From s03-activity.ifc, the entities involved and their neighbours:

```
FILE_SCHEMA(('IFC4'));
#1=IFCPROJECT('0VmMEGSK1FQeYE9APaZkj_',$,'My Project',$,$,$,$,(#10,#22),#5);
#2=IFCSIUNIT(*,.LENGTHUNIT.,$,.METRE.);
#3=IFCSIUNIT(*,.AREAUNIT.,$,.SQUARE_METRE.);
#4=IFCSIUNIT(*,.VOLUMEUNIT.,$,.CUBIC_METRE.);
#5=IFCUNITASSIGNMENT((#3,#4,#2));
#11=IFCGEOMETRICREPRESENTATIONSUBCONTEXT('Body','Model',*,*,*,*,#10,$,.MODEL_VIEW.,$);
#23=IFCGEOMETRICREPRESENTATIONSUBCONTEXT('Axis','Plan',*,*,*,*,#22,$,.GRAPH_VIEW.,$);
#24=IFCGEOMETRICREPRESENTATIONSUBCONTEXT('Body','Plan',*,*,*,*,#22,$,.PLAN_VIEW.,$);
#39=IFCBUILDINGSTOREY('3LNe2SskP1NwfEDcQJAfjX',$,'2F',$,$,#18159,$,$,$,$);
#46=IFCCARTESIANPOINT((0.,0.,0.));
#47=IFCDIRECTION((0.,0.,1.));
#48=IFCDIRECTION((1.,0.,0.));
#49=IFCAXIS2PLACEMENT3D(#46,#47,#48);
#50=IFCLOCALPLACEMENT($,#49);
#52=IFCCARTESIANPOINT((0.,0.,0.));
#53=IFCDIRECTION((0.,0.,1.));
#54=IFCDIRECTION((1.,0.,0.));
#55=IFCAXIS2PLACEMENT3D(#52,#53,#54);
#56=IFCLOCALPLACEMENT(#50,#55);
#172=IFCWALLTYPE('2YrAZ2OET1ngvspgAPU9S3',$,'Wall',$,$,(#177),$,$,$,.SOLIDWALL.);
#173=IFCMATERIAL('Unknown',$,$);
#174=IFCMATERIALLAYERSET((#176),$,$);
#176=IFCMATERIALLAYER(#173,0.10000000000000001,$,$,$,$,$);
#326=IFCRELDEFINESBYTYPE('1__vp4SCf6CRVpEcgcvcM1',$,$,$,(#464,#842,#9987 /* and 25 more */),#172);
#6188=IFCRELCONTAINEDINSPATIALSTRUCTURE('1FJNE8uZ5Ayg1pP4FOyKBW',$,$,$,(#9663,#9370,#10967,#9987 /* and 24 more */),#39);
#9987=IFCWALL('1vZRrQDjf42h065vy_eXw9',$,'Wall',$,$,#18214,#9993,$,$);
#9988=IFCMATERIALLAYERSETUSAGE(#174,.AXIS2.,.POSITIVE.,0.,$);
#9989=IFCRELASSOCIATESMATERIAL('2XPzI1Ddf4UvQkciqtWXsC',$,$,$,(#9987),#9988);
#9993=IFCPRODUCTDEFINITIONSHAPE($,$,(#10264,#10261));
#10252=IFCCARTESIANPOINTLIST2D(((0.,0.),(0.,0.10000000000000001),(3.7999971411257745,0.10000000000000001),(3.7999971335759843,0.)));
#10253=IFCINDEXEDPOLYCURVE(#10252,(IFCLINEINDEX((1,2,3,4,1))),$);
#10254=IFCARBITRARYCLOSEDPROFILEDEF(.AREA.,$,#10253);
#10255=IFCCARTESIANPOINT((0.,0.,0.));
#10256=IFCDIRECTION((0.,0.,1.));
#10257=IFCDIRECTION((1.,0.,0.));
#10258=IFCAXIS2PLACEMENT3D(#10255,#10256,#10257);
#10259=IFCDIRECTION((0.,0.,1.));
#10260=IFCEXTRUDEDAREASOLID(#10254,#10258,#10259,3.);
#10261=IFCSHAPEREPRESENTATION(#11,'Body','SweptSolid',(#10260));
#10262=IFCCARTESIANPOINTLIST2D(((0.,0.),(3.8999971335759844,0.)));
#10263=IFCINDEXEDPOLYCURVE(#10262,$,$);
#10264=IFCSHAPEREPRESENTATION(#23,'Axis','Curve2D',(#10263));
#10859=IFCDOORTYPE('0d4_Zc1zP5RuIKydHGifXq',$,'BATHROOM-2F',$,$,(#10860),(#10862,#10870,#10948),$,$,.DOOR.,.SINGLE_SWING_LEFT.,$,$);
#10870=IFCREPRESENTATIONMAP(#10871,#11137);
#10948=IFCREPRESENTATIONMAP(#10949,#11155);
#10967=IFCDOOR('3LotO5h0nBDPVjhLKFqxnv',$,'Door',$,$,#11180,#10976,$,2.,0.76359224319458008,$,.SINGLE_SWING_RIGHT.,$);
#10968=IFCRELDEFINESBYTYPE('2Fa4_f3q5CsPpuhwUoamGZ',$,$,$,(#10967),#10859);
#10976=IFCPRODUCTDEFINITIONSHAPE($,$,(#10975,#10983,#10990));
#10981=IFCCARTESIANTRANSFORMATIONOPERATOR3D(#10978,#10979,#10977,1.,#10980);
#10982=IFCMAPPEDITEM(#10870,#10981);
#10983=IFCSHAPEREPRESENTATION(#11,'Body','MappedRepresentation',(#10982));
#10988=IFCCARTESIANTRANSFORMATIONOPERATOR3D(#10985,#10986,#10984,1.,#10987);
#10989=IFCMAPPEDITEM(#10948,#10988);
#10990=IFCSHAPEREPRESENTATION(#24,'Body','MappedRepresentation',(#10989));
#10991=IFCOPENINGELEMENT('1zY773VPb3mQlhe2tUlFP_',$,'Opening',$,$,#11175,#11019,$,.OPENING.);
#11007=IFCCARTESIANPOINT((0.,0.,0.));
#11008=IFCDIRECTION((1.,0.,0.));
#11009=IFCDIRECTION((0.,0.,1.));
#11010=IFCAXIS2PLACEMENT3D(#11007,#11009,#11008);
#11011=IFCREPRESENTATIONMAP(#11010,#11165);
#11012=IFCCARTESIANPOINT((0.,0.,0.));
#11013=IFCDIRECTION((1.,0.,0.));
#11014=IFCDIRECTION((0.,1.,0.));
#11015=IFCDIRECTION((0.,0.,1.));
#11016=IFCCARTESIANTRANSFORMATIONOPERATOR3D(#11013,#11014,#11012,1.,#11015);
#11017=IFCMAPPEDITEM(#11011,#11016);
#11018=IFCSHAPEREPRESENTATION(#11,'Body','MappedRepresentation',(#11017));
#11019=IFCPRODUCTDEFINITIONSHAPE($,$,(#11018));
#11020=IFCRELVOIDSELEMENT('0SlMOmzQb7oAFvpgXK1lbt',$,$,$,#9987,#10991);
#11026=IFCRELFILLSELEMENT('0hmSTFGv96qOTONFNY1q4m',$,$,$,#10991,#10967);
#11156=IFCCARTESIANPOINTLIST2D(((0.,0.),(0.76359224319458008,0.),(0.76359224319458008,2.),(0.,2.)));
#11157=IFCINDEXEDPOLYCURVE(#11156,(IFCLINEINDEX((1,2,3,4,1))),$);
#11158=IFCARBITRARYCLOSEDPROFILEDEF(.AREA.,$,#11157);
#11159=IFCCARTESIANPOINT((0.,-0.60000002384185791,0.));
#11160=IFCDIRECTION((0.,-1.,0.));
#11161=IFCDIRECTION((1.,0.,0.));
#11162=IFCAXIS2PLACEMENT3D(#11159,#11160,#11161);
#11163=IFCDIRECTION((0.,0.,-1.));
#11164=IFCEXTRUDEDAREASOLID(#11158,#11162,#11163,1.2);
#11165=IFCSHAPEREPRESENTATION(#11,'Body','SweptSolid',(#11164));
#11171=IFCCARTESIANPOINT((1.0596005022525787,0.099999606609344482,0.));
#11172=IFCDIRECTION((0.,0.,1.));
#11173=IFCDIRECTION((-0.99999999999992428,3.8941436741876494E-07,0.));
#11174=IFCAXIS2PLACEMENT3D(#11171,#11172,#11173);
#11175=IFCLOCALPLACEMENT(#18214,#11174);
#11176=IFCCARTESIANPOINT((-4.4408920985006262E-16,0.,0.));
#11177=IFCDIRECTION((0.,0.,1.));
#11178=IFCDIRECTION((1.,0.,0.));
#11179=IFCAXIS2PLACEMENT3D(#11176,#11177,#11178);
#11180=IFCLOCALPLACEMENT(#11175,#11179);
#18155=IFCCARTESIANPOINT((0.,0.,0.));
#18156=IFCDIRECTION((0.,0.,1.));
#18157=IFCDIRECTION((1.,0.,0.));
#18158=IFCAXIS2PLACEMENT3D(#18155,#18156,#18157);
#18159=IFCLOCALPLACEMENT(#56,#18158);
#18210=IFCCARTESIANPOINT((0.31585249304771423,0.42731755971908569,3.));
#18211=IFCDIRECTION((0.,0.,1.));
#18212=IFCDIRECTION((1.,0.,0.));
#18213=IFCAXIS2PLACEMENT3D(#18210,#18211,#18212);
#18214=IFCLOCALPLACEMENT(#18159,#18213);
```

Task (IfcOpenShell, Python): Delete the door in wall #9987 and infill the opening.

```python
import ifcopenshell
import ifcopenshell.api.feature
import ifcopenshell.api.root
import ifcopenshell.geom
import ifcopenshell.util.shape

model = ifcopenshell.open("s03-activity.ifc")
settings = ifcopenshell.geom.settings()


def volume(element):
    """Net volume in cubic metres, openings subtracted."""
    shape = ifcopenshell.geom.create_shape(settings, element)
    return ifcopenshell.util.shape.get_volume(shape.geometry)


door = model.by_guid("3LotO5h0nBDPVjhLKFqxnv")
opening = door.FillsVoids[0].RelatingOpeningElement
wall = opening.VoidsElements[0].RelatingBuildingElement
before = volume(wall)

ifcopenshell.api.root.remove_product(model, product=door)
ifcopenshell.api.feature.remove_feature(model, feature=opening)

after = volume(wall)

print(f"wall volume {before:.3f} -> {after:.3f} m3")

model.write("s03-activity_v2.ifc")
```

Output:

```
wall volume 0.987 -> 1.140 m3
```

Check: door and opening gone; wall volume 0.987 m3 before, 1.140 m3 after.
